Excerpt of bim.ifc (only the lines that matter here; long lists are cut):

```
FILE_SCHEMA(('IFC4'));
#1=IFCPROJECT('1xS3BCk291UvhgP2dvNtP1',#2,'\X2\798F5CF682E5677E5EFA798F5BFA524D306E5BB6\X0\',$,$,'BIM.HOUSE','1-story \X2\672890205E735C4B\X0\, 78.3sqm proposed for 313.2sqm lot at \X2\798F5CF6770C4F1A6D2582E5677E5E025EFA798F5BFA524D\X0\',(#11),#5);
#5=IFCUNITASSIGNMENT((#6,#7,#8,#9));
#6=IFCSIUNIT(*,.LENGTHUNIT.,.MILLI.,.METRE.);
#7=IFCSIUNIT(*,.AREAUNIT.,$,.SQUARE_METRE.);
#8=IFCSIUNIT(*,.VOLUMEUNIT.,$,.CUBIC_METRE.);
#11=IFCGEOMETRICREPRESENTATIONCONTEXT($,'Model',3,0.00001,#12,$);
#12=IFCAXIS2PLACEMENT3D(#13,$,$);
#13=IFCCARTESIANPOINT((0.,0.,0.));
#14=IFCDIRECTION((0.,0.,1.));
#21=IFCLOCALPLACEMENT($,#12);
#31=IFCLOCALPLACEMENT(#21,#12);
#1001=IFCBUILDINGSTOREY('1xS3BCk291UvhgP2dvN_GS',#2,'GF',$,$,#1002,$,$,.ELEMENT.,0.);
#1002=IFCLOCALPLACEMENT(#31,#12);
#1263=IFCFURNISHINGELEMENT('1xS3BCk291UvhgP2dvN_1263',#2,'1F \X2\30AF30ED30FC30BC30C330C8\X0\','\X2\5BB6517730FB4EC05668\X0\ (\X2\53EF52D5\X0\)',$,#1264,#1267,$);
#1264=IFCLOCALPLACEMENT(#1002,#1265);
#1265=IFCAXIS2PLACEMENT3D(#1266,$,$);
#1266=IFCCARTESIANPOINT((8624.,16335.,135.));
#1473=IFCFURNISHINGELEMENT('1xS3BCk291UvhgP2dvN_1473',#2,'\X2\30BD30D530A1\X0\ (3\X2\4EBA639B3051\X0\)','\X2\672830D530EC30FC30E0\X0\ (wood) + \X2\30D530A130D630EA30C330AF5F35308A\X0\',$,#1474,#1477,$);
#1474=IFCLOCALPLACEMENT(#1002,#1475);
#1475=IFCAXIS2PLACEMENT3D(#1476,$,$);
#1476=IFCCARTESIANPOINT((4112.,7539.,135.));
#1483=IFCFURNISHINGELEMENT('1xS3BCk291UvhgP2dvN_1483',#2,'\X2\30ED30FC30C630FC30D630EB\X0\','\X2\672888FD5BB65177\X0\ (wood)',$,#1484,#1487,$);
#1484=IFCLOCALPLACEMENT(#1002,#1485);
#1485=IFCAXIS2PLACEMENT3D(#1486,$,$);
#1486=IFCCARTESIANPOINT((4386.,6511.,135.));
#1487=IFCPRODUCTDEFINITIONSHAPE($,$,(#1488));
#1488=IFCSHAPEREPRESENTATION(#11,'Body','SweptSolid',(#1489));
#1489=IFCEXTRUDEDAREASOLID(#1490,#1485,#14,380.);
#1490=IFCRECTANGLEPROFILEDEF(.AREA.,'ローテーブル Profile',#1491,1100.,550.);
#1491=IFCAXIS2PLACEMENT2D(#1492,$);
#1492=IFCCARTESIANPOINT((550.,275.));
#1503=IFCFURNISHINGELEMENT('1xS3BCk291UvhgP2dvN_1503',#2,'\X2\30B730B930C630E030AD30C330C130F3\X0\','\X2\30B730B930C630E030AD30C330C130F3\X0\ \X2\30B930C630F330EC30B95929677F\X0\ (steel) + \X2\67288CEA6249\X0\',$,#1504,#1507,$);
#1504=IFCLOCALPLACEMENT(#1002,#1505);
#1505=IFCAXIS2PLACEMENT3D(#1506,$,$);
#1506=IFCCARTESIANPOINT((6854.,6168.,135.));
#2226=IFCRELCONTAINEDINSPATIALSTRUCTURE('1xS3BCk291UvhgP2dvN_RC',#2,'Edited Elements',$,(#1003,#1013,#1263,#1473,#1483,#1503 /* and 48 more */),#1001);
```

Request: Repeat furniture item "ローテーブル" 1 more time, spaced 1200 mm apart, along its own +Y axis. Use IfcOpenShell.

```python
import ifcopenshell
import ifcopenshell.api.geometry
import ifcopenshell.api.root
import ifcopenshell.util.element
import ifcopenshell.util.placement

model = ifcopenshell.open("bim.ifc")


def reuse_history(source, copy):
    """copy_class also copies each property set's owner history, people and application; keep the originals."""
    for rel in copy.IsDefinedBy:
        if rel.is_a("IfcRelDefinesByProperties") and (history := rel.RelatingPropertyDefinition.OwnerHistory):
            rel.RelatingPropertyDefinition.OwnerHistory = source.OwnerHistory
            ifcopenshell.util.element.remove_deep2(model, history)


source = model.by_guid("1xS3BCk291UvhgP2dvN_1483")
base = ifcopenshell.util.placement.get_local_placement(source.ObjectPlacement)
step = base[:3, 1] * 1200.0

for i in range(1, 2):
    copy = ifcopenshell.api.root.copy_class(model, product=source)
    copy.Representation = ifcopenshell.util.element.copy_deep(
        model, source.Representation, exclude=["IfcGeometricRepresentationContext", "IfcRepresentationMap"]
    )
    reuse_history(source, copy)
    matrix = base.copy()
    matrix[:3, 3] += i * step
    print("added at", matrix[:3, 3].round(3) + 0.0)
    ifcopenshell.api.geometry.edit_object_placement(model, product=copy, matrix=matrix, is_si=False)

model.write("bim_rev.ifc")
```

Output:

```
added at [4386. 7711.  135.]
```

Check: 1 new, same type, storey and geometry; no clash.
